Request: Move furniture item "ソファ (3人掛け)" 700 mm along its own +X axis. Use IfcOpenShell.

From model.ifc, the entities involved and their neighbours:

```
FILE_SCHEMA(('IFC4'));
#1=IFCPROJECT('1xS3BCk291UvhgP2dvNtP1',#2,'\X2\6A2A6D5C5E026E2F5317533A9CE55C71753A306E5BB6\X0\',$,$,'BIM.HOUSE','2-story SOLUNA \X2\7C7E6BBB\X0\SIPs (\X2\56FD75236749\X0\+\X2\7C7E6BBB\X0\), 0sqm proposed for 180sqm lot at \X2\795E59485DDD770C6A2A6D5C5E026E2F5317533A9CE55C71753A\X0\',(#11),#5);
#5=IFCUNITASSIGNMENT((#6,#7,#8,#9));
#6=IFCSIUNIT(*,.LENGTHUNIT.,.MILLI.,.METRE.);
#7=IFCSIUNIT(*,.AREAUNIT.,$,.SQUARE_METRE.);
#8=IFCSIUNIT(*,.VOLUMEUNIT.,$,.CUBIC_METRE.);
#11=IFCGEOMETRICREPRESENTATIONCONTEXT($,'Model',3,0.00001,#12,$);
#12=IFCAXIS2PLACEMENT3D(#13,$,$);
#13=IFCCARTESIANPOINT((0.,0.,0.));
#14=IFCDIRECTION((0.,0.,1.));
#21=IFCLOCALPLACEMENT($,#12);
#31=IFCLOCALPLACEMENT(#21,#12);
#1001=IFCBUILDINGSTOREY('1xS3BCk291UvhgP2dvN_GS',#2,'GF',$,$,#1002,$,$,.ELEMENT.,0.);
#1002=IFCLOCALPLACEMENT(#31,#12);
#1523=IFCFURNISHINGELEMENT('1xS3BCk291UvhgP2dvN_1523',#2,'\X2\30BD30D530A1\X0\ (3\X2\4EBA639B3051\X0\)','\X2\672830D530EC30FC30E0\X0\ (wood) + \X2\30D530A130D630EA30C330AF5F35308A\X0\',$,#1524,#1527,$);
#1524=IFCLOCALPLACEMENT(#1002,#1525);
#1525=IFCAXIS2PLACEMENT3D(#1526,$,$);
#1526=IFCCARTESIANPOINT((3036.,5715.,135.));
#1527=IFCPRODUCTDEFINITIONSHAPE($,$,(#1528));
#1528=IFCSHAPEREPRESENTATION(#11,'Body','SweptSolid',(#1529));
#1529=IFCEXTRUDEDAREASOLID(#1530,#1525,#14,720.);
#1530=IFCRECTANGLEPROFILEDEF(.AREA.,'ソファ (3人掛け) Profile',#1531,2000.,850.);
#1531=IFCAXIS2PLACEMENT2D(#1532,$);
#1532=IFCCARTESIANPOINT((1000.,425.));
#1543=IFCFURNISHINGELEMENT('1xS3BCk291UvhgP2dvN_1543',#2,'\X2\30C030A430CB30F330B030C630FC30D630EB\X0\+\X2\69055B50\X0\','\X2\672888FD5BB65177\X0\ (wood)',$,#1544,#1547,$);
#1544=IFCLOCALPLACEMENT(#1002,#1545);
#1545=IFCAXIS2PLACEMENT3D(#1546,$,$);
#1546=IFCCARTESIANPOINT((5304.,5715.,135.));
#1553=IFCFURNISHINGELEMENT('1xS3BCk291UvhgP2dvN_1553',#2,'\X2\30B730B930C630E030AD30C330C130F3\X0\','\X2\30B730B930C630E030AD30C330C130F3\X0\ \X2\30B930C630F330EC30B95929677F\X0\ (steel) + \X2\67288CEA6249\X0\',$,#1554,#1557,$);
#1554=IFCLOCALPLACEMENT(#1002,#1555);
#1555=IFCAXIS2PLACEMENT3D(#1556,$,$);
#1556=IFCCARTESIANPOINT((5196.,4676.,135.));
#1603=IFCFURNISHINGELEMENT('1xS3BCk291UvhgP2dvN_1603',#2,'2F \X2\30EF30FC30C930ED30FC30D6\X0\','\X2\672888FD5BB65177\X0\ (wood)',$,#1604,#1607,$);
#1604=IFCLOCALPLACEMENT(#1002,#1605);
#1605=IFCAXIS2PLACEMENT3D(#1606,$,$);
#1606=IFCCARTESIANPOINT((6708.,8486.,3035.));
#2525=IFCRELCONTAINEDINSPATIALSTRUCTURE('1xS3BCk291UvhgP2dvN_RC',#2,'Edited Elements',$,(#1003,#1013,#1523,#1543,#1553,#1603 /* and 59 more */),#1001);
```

```python
import ifcopenshell
import ifcopenshell.api.geometry
import ifcopenshell.util.placement

model = ifcopenshell.open("model.ifc")

item = model.by_id(1523)
matrix = ifcopenshell.util.placement.get_local_placement(item.ObjectPlacement)
matrix[:3, 3] += matrix[:3, 0] * 700.0
ifcopenshell.api.geometry.edit_object_placement(model, product=item, matrix=matrix, is_si=False)

print(ifcopenshell.util.placement.get_local_placement(item.ObjectPlacement).round(3) + 0.0)

model.write("model_edited.ifc")
```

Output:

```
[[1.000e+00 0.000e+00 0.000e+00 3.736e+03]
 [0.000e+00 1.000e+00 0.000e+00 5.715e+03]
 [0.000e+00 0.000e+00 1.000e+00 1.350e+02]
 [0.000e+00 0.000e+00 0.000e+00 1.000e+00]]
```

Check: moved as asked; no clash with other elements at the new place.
